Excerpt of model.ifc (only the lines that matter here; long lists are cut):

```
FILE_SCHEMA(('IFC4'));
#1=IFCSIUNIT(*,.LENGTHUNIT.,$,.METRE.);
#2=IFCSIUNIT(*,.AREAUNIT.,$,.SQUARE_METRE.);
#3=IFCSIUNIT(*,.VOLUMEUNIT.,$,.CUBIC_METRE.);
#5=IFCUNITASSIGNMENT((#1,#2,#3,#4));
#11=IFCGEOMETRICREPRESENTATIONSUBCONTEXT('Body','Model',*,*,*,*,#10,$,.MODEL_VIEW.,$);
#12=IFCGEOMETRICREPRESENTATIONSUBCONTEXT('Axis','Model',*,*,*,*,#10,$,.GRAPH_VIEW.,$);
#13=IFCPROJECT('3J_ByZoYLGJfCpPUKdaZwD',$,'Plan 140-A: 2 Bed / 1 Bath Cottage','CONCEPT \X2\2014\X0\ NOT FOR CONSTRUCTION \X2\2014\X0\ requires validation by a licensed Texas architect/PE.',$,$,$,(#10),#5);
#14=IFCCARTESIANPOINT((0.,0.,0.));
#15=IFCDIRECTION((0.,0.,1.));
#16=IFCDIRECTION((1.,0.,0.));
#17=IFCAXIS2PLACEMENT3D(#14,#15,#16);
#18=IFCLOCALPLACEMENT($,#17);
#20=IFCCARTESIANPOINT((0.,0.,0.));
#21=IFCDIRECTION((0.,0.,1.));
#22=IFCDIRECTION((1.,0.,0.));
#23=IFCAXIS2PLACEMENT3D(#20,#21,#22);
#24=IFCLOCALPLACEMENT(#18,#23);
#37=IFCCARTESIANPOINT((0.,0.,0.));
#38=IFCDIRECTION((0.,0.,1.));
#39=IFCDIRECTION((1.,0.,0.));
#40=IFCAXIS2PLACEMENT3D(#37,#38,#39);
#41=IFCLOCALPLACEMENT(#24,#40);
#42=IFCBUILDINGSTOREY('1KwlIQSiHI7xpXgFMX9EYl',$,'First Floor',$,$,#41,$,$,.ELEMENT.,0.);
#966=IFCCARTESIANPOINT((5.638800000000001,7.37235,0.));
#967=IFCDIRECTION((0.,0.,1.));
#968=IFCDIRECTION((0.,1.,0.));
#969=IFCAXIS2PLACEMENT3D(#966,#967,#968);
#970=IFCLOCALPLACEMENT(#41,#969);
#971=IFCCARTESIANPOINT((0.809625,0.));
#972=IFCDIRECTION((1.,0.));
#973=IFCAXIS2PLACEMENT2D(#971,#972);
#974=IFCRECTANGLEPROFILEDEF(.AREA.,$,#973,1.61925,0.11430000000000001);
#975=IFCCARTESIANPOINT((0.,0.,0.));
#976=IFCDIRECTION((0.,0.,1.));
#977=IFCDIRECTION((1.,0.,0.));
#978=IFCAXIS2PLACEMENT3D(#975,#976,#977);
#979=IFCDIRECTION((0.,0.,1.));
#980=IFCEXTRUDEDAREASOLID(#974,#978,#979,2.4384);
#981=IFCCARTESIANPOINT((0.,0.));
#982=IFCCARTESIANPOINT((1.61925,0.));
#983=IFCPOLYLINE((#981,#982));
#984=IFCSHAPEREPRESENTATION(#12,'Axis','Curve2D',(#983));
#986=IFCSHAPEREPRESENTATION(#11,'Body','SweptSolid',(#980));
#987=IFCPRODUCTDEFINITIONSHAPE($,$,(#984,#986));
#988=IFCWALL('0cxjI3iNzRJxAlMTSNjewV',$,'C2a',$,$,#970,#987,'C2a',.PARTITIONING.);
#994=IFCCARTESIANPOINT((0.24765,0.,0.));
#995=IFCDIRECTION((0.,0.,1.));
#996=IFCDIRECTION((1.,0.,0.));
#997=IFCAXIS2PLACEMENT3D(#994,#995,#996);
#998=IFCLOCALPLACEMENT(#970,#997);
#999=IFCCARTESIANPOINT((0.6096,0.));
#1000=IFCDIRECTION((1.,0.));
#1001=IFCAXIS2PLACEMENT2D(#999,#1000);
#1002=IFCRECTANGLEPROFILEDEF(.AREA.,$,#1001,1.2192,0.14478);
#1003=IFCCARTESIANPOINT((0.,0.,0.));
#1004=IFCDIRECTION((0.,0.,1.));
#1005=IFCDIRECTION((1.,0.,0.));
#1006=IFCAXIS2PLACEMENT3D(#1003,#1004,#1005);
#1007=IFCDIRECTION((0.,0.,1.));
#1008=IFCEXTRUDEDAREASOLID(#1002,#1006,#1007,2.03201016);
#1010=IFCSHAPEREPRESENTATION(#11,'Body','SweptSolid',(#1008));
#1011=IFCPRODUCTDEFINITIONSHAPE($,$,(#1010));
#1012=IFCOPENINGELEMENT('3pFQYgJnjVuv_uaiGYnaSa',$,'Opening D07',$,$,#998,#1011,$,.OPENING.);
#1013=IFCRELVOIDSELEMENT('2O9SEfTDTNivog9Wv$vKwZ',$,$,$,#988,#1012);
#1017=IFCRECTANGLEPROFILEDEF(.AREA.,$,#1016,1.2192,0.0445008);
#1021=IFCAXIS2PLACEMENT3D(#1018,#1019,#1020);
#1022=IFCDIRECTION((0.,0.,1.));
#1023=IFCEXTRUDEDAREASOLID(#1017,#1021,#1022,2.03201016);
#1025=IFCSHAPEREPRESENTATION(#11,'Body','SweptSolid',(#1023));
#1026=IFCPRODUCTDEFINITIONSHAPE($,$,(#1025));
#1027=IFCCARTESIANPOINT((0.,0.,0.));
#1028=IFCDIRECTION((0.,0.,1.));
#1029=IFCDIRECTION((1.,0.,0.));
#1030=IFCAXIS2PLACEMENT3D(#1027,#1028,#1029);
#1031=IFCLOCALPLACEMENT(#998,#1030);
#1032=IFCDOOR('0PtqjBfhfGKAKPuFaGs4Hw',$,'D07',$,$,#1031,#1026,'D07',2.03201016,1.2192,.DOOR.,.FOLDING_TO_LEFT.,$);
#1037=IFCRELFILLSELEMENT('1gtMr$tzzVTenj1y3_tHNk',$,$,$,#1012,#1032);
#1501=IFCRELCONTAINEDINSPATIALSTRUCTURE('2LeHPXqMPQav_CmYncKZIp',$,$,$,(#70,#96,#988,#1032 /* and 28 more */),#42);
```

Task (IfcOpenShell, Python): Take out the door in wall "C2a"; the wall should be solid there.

```python
import ifcopenshell
import ifcopenshell.api.feature
import ifcopenshell.api.root
import ifcopenshell.geom
import ifcopenshell.util.shape

model = ifcopenshell.open("model.ifc")
settings = ifcopenshell.geom.settings()


def volume(element):
    """Net volume in cubic metres, openings subtracted."""
    shape = ifcopenshell.geom.create_shape(settings, element)
    return ifcopenshell.util.shape.get_volume(shape.geometry)


door = model.by_id(1032)
opening = door.FillsVoids[0].RelatingOpeningElement
wall = opening.VoidsElements[0].RelatingBuildingElement
before = volume(wall)

ifcopenshell.api.root.remove_product(model, product=door)
ifcopenshell.api.feature.remove_feature(model, feature=opening)

after = volume(wall)

print(f"wall volume {before:.3f} -> {after:.3f} m3")

model.write("model_updated.ifc")
```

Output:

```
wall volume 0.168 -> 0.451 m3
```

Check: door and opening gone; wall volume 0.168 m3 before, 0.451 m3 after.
